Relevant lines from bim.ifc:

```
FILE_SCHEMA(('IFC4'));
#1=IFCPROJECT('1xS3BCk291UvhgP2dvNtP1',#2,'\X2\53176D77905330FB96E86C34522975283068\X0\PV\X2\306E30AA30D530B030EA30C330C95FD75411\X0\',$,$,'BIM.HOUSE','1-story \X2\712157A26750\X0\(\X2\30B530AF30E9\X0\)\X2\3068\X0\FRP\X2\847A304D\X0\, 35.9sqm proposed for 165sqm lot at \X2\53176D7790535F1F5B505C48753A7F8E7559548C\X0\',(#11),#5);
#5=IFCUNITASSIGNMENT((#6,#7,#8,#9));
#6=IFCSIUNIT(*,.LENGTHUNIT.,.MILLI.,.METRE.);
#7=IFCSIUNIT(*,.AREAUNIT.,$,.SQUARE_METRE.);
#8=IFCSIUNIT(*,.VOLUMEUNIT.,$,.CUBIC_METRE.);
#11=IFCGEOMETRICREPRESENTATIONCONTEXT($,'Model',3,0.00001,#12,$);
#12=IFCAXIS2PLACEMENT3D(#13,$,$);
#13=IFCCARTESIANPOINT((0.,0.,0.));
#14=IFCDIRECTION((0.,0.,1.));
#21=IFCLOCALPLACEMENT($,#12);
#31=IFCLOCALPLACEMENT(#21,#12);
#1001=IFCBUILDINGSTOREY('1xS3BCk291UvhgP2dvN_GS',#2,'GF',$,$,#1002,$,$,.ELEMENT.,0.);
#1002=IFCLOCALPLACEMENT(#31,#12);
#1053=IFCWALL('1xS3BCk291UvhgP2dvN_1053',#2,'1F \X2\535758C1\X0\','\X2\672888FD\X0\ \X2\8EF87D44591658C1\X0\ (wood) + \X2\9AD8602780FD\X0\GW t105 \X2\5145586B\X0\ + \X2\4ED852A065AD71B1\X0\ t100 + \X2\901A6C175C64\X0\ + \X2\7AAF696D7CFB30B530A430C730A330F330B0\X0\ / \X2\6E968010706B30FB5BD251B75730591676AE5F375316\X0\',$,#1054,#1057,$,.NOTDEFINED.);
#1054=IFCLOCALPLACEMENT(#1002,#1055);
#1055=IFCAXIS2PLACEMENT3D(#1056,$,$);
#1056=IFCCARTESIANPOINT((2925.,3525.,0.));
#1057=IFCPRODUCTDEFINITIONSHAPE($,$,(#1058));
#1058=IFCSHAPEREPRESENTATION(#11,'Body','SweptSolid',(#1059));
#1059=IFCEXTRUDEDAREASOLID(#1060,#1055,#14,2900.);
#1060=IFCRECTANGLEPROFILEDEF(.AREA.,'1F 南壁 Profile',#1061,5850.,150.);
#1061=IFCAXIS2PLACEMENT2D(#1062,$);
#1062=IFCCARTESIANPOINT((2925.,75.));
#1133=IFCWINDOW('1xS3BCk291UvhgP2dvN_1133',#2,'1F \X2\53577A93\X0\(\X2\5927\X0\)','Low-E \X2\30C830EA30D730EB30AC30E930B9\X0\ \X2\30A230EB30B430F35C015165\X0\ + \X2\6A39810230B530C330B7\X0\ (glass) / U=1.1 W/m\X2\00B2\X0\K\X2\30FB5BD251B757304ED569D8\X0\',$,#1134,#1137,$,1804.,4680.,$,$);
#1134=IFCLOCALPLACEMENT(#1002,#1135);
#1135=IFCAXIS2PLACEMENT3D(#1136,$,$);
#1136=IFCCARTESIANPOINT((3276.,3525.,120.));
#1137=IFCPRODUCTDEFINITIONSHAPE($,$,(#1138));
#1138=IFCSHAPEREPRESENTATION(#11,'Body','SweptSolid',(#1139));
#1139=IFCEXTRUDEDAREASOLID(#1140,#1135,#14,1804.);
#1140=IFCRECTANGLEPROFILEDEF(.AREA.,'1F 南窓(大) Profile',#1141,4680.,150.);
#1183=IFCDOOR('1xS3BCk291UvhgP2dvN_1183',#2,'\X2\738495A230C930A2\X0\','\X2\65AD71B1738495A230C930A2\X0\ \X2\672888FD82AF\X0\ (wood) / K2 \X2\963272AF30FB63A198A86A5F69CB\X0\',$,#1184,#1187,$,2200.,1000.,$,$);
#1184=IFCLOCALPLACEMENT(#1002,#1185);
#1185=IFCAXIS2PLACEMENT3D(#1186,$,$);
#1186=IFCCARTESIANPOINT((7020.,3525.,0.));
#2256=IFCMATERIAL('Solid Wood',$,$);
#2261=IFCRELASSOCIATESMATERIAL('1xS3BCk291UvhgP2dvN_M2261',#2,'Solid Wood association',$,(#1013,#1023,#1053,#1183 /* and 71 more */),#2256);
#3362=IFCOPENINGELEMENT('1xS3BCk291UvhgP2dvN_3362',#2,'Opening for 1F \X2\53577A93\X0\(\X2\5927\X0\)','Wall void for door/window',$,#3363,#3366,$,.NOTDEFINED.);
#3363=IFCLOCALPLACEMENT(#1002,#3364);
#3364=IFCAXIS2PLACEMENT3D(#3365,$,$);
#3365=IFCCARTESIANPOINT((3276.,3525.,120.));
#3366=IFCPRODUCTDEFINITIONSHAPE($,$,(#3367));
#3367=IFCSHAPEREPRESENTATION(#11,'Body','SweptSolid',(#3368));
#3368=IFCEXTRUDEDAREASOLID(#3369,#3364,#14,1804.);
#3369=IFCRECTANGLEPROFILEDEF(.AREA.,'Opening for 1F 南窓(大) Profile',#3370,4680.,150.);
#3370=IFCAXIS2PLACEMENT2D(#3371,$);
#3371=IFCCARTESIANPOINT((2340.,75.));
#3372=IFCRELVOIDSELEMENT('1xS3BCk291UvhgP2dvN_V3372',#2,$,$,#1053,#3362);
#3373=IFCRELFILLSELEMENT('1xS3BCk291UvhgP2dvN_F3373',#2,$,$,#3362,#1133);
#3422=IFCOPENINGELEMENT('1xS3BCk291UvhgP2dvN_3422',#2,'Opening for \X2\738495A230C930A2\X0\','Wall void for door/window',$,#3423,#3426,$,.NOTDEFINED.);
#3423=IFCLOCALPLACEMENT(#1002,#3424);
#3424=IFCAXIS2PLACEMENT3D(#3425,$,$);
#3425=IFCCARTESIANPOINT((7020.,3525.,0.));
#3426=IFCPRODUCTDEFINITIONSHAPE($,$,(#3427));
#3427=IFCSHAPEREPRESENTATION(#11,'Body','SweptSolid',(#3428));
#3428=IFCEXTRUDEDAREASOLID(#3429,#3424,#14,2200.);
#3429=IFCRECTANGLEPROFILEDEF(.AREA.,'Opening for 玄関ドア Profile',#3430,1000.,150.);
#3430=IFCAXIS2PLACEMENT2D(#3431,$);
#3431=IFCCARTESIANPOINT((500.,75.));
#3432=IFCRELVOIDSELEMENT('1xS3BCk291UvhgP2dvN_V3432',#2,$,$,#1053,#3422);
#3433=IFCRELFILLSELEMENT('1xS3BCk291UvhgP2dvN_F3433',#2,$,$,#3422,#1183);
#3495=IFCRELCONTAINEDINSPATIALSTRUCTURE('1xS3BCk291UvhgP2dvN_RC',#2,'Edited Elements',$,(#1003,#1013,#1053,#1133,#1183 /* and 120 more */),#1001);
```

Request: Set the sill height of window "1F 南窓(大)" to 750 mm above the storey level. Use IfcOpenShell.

```python
import numpy as np
import ifcopenshell
import ifcopenshell.api.geometry
import ifcopenshell.geom
import ifcopenshell.util.element
import ifcopenshell.util.placement
import ifcopenshell.util.shape
import ifcopenshell.util.unit

model = ifcopenshell.open("bim.ifc")
unit_scale = ifcopenshell.util.unit.calculate_unit_scale(model)

window = model.by_guid("1xS3BCk291UvhgP2dvN_1133")
opening = window.FillsVoids[0].RelatingOpeningElement
storey = ifcopenshell.util.element.get_container(window, ifc_class="IfcBuildingStorey")
level = ifcopenshell.util.placement.get_local_placement(storey.ObjectPlacement)[2, 3]

# The opening's origin need not be at the sill, so measure its lowest point.
shape = ifcopenshell.geom.create_shape(ifcopenshell.geom.settings(), opening)
bottom = ifcopenshell.util.shape.get_shape_bottom_elevation(shape, shape.geometry) / unit_scale
dz = level + 0.75 / unit_scale - bottom

shift = np.array([0.0, 0.0, dz])
# The window is not placed relative to its opening, so move both.
for product in (opening, window):
    matrix = ifcopenshell.util.placement.get_local_placement(product.ObjectPlacement)
    matrix[:3, 3] += shift
    ifcopenshell.api.geometry.edit_object_placement(model, product=product, matrix=matrix, is_si=False)

print(f"moved by {dz * unit_scale:+.3f} m")

model.write("bim_updated.ifc")
```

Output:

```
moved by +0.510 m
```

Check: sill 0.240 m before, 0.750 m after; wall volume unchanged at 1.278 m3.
